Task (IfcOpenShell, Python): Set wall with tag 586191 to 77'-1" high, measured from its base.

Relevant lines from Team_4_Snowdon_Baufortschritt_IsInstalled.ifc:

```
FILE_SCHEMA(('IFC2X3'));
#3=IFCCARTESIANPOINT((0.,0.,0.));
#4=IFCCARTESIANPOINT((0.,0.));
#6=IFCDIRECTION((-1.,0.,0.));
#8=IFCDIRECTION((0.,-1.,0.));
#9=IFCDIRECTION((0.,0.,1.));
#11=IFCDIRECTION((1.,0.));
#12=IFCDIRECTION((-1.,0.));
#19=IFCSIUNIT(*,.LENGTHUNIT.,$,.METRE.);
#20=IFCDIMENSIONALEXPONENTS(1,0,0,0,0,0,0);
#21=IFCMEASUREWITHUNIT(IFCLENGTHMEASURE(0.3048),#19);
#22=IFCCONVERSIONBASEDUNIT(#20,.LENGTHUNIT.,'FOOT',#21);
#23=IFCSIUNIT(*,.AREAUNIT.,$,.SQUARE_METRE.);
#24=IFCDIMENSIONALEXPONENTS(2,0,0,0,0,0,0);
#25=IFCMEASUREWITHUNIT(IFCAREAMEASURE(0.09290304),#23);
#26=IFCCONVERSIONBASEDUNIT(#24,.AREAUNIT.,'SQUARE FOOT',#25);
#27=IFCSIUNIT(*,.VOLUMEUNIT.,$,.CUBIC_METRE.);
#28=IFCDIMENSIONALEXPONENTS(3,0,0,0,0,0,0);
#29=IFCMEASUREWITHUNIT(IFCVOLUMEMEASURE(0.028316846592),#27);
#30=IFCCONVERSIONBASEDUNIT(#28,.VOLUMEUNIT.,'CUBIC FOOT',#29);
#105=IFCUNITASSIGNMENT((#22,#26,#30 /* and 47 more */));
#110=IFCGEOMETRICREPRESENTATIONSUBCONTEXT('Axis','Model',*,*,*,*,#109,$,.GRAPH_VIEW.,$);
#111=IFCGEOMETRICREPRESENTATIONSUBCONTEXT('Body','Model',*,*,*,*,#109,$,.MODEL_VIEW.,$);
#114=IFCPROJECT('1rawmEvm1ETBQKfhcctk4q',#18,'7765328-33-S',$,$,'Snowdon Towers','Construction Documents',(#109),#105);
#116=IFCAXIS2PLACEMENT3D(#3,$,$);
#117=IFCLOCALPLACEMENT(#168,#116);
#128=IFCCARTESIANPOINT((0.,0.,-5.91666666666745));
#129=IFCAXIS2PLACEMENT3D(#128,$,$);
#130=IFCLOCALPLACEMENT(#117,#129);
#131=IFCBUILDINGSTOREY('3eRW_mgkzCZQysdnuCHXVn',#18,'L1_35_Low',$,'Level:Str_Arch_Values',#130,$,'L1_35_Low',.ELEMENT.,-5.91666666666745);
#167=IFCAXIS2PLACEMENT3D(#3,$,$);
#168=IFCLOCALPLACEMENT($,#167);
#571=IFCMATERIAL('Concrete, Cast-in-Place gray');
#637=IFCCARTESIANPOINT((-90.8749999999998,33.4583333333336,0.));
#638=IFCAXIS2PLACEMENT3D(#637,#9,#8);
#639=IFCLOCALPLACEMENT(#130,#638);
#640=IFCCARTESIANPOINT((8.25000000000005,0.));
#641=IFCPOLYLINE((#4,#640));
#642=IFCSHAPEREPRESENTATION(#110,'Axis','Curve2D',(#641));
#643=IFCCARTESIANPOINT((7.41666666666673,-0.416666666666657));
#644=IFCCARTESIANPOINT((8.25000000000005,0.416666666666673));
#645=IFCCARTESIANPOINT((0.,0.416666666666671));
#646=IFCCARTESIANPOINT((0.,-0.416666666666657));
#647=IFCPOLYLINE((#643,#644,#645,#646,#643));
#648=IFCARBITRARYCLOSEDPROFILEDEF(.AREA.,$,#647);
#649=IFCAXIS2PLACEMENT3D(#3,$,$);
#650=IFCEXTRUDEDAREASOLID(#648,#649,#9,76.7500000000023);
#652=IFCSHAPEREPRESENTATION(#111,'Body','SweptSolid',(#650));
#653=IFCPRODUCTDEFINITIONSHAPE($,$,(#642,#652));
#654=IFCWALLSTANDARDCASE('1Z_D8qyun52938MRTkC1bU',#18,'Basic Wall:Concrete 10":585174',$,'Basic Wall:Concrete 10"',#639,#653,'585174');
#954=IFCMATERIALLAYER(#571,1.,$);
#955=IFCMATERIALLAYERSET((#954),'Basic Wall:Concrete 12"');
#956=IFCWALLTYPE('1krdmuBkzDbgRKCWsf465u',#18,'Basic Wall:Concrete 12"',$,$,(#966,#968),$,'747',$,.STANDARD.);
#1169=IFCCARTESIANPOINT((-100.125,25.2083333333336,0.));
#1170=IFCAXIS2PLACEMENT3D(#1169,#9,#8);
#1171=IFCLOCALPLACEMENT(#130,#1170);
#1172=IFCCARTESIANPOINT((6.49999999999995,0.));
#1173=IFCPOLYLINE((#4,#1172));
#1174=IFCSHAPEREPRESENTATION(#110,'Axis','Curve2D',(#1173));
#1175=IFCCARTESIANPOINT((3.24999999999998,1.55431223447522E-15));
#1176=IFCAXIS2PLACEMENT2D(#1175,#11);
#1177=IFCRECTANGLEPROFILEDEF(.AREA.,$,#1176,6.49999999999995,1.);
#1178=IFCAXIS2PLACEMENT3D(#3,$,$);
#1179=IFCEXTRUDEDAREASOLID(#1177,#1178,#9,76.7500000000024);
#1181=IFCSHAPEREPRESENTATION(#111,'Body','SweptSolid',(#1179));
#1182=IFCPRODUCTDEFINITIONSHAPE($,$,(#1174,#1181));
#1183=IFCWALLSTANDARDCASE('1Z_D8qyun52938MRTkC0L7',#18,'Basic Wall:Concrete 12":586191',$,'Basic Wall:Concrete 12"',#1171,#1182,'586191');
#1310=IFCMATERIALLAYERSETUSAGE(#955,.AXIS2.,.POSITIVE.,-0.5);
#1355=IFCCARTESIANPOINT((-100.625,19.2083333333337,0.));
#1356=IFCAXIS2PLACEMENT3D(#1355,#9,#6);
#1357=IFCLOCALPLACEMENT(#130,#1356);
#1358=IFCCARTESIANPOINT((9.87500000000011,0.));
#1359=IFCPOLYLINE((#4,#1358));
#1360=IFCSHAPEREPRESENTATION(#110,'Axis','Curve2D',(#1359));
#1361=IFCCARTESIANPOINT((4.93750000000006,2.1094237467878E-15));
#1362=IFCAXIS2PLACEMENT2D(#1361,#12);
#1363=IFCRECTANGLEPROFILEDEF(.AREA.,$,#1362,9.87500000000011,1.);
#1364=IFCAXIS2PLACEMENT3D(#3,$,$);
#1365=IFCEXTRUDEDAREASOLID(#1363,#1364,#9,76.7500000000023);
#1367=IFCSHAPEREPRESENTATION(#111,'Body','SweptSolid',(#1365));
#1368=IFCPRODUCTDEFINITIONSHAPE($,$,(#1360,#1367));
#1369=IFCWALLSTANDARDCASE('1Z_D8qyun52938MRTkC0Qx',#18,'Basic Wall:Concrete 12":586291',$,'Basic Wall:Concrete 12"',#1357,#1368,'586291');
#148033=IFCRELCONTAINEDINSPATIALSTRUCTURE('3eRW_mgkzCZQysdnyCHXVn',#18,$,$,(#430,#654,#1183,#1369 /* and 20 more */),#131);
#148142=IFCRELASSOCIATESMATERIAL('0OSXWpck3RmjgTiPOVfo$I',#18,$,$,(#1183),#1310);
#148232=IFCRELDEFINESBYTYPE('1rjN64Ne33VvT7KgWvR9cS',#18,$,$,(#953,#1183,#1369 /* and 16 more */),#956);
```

```python
import ifcopenshell
import ifcopenshell.geom
import ifcopenshell.util.representation
import ifcopenshell.util.shape
import ifcopenshell.util.unit

model = ifcopenshell.open("Team_4_Snowdon_Baufortschritt_IsInstalled.ifc")
unit_scale = ifcopenshell.util.unit.calculate_unit_scale(model)
settings = ifcopenshell.geom.settings()


def volume(element):
    """Net volume in cubic metres, openings subtracted."""
    shape = ifcopenshell.geom.create_shape(settings, element)
    return ifcopenshell.util.shape.get_volume(shape.geometry)


wall = model.by_guid("1Z_D8qyun52938MRTkC0L7")
before = volume(wall)

body = ifcopenshell.util.representation.get_representation(wall, "Model", "Body")
solid = body.Items[0]
old_height = solid.Depth
solid.Depth = 925 * 0.0254 / unit_scale
after = volume(wall)

print(f"height {old_height:g} -> {solid.Depth:g}, volume {before:.3f} -> {after:.3f} m3")

model.write("Team_4_Snowdon_Baufortschritt_IsInstalled_edited.ifc")
```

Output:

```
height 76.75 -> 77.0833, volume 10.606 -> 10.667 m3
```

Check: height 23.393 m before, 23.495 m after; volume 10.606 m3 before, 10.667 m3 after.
